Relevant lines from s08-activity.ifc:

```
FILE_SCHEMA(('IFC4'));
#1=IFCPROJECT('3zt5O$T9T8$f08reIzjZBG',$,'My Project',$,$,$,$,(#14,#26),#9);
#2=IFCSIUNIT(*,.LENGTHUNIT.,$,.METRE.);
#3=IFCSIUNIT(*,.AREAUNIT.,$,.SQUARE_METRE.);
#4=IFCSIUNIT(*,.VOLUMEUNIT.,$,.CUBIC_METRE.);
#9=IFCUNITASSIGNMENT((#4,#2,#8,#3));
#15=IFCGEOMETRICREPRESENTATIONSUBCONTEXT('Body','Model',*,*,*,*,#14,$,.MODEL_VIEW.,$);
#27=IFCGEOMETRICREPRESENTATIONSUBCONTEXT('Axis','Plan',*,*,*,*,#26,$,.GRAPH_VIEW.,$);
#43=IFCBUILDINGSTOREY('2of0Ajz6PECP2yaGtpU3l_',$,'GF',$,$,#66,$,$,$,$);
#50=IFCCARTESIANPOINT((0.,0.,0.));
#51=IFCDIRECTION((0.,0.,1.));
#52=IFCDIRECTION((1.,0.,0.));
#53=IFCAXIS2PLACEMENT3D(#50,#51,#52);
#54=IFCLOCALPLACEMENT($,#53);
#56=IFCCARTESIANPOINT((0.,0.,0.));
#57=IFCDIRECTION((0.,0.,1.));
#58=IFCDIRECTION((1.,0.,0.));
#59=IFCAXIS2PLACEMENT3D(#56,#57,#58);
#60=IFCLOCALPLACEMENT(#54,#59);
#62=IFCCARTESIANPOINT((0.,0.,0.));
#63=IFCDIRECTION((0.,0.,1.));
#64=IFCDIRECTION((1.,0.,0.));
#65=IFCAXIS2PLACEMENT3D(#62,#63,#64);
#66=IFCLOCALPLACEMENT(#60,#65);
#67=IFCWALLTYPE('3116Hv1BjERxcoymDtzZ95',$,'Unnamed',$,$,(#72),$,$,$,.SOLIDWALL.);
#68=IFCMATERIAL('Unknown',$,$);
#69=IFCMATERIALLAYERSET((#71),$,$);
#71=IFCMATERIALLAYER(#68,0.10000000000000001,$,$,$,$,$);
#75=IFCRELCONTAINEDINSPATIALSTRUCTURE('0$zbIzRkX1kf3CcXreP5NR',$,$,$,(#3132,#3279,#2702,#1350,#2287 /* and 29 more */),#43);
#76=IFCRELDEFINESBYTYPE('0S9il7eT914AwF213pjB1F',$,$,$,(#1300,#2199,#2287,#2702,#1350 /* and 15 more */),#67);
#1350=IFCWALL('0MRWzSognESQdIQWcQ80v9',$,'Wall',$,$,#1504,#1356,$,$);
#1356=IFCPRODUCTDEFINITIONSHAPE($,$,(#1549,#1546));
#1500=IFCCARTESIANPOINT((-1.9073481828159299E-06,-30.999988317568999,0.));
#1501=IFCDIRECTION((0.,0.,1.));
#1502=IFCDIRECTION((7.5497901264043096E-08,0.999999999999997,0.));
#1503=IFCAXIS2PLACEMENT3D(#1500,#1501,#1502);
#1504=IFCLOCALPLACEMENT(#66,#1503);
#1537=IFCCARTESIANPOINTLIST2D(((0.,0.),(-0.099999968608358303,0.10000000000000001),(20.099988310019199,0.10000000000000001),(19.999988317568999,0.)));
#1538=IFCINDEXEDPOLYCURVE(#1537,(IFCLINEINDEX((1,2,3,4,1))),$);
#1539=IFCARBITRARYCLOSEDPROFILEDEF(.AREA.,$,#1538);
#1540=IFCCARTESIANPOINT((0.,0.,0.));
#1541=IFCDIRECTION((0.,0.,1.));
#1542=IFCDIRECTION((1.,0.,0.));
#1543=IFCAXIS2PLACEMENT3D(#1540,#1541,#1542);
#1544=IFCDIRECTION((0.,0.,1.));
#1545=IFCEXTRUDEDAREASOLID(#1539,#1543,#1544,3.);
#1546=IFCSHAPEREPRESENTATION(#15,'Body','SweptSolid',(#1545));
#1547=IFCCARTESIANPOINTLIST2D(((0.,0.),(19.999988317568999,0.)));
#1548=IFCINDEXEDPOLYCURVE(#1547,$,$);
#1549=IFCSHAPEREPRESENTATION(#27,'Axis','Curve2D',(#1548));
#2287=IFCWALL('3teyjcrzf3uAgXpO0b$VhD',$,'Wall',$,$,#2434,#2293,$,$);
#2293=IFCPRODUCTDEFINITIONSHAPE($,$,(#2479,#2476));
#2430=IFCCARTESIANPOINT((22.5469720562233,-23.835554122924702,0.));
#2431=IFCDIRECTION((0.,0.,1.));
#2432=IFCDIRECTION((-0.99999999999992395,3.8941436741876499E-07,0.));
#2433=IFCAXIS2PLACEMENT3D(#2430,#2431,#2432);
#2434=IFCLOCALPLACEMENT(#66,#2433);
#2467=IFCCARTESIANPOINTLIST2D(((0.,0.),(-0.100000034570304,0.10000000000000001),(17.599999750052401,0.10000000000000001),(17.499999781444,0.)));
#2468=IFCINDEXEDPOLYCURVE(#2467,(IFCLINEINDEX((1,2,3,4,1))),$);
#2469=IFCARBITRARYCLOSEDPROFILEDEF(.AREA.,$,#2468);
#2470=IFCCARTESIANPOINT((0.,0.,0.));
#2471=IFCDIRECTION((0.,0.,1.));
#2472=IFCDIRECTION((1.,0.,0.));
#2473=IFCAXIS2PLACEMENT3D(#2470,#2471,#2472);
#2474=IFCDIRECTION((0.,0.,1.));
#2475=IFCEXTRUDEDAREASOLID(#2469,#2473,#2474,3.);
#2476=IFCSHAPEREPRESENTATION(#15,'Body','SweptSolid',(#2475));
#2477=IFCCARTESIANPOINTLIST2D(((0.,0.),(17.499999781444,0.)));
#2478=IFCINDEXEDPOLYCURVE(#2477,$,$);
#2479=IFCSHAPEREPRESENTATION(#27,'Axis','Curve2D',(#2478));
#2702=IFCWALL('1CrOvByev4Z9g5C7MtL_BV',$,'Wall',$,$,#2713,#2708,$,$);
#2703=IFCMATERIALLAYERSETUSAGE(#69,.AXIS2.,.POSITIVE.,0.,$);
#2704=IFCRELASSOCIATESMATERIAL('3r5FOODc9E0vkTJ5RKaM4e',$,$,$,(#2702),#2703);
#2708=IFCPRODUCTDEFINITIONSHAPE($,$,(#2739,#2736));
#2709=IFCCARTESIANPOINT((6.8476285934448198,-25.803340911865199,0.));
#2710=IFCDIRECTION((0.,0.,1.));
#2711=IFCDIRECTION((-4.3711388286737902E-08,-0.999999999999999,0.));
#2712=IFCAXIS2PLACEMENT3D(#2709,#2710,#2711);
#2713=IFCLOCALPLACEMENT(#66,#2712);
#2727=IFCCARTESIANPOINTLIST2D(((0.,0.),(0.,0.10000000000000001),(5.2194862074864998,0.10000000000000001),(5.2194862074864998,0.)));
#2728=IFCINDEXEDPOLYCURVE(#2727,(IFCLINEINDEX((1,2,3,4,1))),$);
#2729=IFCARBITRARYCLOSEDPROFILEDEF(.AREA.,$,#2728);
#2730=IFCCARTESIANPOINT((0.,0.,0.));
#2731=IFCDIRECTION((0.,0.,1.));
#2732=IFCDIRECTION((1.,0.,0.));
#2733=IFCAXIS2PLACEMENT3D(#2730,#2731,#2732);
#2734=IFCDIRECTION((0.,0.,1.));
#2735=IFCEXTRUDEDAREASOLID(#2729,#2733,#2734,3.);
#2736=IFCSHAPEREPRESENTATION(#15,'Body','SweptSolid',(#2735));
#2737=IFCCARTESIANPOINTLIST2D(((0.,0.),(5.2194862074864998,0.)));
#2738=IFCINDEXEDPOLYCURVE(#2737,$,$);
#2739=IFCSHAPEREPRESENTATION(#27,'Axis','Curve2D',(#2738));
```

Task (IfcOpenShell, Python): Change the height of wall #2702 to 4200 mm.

```python
import ifcopenshell
import ifcopenshell.geom
import ifcopenshell.util.representation
import ifcopenshell.util.shape

model = ifcopenshell.open("s08-activity.ifc")
settings = ifcopenshell.geom.settings()


def volume(element):
    """Net volume in cubic metres, openings subtracted."""
    shape = ifcopenshell.geom.create_shape(settings, element)
    return ifcopenshell.util.shape.get_volume(shape.geometry)


wall = model.by_guid("1CrOvByev4Z9g5C7MtL_BV")
before = volume(wall)

body = ifcopenshell.util.representation.get_representation(wall, "Model", "Body")
solid = body.Items[0]
old_height = solid.Depth
solid.Depth = 4.2
after = volume(wall)

print(f"height {old_height:g} -> {solid.Depth:g}, volume {before:.3f} -> {after:.3f} m3")

model.write("s08-activity-out.ifc")
```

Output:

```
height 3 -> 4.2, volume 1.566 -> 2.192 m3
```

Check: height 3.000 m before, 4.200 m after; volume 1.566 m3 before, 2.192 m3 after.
